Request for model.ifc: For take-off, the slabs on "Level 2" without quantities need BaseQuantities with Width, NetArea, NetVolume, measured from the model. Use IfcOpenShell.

First a look at what the model holds.

```python
import ifcopenshell
import ifcopenshell.util.element
import ifcopenshell.util.unit

model = ifcopenshell.open("model.ifc")
print(model.schema)
for unit_type in ("LENGTHUNIT", "AREAUNIT", "VOLUMEUNIT"):
    print(unit_type, ifcopenshell.util.unit.calculate_unit_scale(model, unit_type))
storey = next(s for s in model.by_type("IfcBuildingStorey") if s.Name == "Level 2")
slabs = [e for e in ifcopenshell.util.element.get_decomposition(storey) if e.is_a("IfcSlab")]
for e in sorted(slabs, key=lambda e: e.id()):
    print(e.id(), e.is_a(), e.Name, list(ifcopenshell.util.element.get_psets(e, qtos_only=True)), sep=" | ")
```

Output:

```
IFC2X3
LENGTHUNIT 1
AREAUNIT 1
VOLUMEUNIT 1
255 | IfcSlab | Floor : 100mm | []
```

```python
import ifcopenshell
import ifcopenshell.api.pset
import ifcopenshell.geom
import ifcopenshell.util.element
import ifcopenshell.util.shape
import ifcopenshell.util.unit

model = ifcopenshell.open("model.ifc")
unit_scale = ifcopenshell.util.unit.calculate_unit_scale(model)
area_scale = ifcopenshell.util.unit.calculate_unit_scale(model, "AREAUNIT")
volume_scale = ifcopenshell.util.unit.calculate_unit_scale(model, "VOLUMEUNIT")
settings = ifcopenshell.geom.settings()

storey = next(s for s in model.by_type("IfcBuildingStorey") if s.Name == "Level 2")
slabs = [e for e in ifcopenshell.util.element.get_decomposition(storey) if e.is_a("IfcSlab")]

for e in sorted(slabs, key=lambda e: e.id()):
    if ifcopenshell.util.element.get_psets(e, qtos_only=True, should_inherit=False):
        continue
    # Geometry comes back in metres, in the element's own axes.
    shape = ifcopenshell.geom.create_shape(settings, e)
    values = {
        "Width": ifcopenshell.util.shape.get_z(shape.geometry) / unit_scale,
        "NetArea": ifcopenshell.util.shape.get_footprint_area(shape.geometry) / area_scale,
        "NetVolume": ifcopenshell.util.shape.get_volume(shape.geometry) / volume_scale,
    }
    qto = ifcopenshell.api.pset.add_qto(model, product=e, name="BaseQuantities")
    ifcopenshell.api.pset.edit_qto(model, qto=qto, properties=values)
    print(e.id(), {k: round(v, 3) for k, v in values.items()})

model.write("model-out.ifc")
```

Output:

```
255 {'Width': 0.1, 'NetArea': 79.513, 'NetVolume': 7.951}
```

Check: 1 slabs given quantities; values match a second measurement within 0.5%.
